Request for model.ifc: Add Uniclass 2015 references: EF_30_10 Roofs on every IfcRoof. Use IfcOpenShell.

First a look at what the model holds.

```python
import ifcopenshell

model = ifcopenshell.open("model.ifc")
print(model.schema)
print("classifications:", [c.Name for c in model.by_type("IfcClassification")])
for ifc_class in ("IfcDoor", "IfcRoof", "IfcStair", "IfcWall", "IfcWindow"):
    print(ifc_class, len(model.by_type(ifc_class)))
```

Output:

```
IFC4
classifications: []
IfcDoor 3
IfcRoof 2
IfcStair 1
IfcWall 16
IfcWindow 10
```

```python
import ifcopenshell
import ifcopenshell.api.classification

model = ifcopenshell.open("model.ifc")

system = ifcopenshell.api.classification.add_classification(model, classification="Uniclass 2015")

codes = {
    "IfcRoof": ("EF_30_10", "Roofs"),
}
for ifc_class, (code, name) in codes.items():
    products = model.by_type(ifc_class)
    ifcopenshell.api.classification.add_reference(
        model, products=products, classification=system, identification=code, name=name
    )
    print(code, len(products))

model.write("model_edited.ifc")
```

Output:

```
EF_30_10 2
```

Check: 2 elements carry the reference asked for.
